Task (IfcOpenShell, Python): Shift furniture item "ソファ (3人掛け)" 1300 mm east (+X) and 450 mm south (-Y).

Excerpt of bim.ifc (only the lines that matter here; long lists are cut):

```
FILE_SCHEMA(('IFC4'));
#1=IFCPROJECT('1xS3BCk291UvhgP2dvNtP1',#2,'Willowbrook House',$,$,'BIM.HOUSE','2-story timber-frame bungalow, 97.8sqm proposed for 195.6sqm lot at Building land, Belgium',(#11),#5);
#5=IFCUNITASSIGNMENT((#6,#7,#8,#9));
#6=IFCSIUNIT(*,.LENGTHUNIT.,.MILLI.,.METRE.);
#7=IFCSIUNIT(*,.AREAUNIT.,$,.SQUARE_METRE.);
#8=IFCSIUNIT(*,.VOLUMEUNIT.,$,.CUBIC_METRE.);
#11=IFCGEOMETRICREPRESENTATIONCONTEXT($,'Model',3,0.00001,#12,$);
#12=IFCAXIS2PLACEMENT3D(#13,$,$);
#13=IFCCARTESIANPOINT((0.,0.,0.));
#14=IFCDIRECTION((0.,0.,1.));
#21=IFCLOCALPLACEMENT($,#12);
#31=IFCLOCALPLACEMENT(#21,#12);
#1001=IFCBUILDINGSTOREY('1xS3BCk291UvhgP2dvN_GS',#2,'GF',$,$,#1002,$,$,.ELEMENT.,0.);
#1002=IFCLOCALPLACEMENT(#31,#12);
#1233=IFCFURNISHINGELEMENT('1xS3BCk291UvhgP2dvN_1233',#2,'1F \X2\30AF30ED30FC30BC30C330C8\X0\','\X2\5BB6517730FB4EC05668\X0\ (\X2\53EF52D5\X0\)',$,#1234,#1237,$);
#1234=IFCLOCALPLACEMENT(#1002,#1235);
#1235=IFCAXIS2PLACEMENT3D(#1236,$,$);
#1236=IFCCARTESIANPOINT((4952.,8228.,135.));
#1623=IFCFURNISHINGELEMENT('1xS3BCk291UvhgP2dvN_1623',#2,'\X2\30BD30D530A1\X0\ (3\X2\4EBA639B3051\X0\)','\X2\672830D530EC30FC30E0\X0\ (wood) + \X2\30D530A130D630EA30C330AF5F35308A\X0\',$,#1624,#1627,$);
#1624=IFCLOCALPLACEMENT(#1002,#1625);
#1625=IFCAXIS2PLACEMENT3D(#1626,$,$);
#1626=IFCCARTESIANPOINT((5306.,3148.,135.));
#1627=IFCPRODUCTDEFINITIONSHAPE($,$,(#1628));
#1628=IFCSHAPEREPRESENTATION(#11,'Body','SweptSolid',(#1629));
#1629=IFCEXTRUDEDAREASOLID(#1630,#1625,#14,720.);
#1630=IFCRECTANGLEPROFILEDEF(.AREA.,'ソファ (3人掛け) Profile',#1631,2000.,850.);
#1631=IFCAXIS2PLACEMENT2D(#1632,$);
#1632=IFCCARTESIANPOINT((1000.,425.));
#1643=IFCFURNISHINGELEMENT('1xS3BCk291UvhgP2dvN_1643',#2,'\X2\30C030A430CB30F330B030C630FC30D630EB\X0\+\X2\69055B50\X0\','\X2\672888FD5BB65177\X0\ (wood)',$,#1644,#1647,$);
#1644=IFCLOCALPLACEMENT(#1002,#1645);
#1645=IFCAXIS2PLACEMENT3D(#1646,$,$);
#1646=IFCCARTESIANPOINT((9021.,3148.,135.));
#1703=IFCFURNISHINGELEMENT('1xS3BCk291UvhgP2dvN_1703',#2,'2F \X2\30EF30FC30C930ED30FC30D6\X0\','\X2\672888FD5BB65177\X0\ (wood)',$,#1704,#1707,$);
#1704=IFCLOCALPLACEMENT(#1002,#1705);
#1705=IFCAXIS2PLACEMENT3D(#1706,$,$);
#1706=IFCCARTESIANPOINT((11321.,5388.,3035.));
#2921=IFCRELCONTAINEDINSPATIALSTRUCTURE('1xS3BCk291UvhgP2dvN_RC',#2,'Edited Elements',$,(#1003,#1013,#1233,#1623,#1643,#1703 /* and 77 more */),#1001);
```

```python
import ifcopenshell
import ifcopenshell.api.geometry
import ifcopenshell.util.placement
import ifcopenshell.util.unit

model = ifcopenshell.open("bim.ifc")
unit_scale = ifcopenshell.util.unit.calculate_unit_scale(model)

item = model.by_guid("1xS3BCk291UvhgP2dvN_1623")
matrix = ifcopenshell.util.placement.get_local_placement(item.ObjectPlacement)
matrix[0, 3] += 1.3 / unit_scale
matrix[1, 3] -= 0.45 / unit_scale
ifcopenshell.api.geometry.edit_object_placement(model, product=item, matrix=matrix, is_si=False)

print(ifcopenshell.util.placement.get_local_placement(item.ObjectPlacement).round(3) + 0.0)

model.write("bim_v2.ifc")
```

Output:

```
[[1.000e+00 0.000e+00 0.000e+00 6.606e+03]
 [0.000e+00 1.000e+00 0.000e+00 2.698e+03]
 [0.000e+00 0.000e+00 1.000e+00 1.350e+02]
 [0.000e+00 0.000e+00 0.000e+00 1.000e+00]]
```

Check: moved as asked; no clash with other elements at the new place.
